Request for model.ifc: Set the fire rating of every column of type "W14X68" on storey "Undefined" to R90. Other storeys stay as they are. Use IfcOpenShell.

First a look at what the model holds.

```python
import ifcopenshell
import ifcopenshell.util.element

model = ifcopenshell.open("model.ifc")
print(model.schema)
storey = next(s for s in model.by_type("IfcBuildingStorey") if s.Name == "Undefined")
columns = [e for e in ifcopenshell.util.element.get_decomposition(storey) if e.is_a("IfcColumn")]
seen = {}
for e in columns:
    element_type = ifcopenshell.util.element.get_type(e)
    key = (element_type.Name if element_type != e and element_type else None, ifcopenshell.util.element.get_pset(e, "Pset_ColumnCommon", "FireRating"))
    seen[key] = seen.get(key, 0) + 1
for (name, value), count in sorted(seen.items(), key=str):
    print(count, "x", name, "|", value)
```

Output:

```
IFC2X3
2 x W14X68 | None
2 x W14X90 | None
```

```python
import ifcopenshell
import ifcopenshell.api.pset
import ifcopenshell.util.element

model = ifcopenshell.open("model.ifc")

storey = next(s for s in model.by_type("IfcBuildingStorey") if s.Name == "Undefined")
columns = [e for e in ifcopenshell.util.element.get_decomposition(storey) if e.is_a("IfcColumn")]

count = 0
for e in columns:
    element_type = ifcopenshell.util.element.get_type(e)
    if element_type in (None, e) or element_type.Name != "W14X68":
        continue
    found = ifcopenshell.util.element.get_pset(e, "Pset_ColumnCommon", should_inherit=False)
    if found:
        pset = model.by_id(found["id"])
        if len(ifcopenshell.util.element.get_elements_by_pset(pset)) > 1:
            pset = ifcopenshell.api.pset.unshare_pset(model, products=[e], pset=pset)[0]
    else:
        pset = ifcopenshell.api.pset.add_pset(model, product=e, name="Pset_ColumnCommon")
    ifcopenshell.api.pset.edit_pset(model, pset=pset, properties={"FireRating": "R90"})
    count += 1

print(count, "columns updated")

model.write("model_v2.ifc")
```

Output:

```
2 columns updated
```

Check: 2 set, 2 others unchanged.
